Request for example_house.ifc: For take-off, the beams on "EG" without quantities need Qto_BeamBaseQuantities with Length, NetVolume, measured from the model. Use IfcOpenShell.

First a look at what the model holds.

```python
import ifcopenshell
import ifcopenshell.util.element
import ifcopenshell.util.unit

model = ifcopenshell.open("example_house.ifc")
print(model.schema)
for unit_type in ("LENGTHUNIT", "AREAUNIT", "VOLUMEUNIT"):
    print(unit_type, ifcopenshell.util.unit.calculate_unit_scale(model, unit_type))
storey = next(s for s in model.by_type("IfcBuildingStorey") if s.Name == "EG")
beams = [e for e in ifcopenshell.util.element.get_decomposition(storey) if e.is_a("IfcBeam")]
for e in sorted(beams, key=lambda e: e.id()):
    print(e.id(), e.is_a(), e.Name, list(ifcopenshell.util.element.get_psets(e, qtos_only=True)), sep=" | ")
```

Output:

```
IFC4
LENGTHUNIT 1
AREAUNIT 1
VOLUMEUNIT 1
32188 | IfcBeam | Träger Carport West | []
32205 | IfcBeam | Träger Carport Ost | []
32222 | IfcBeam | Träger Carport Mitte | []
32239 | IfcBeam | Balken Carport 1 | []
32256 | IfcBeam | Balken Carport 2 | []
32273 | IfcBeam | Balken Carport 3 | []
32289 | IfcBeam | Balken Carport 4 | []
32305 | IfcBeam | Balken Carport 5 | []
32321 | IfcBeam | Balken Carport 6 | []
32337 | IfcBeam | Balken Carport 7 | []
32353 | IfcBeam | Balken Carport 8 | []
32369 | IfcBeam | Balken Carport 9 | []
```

```python
import ifcopenshell
import ifcopenshell.api.pset
import ifcopenshell.geom
import ifcopenshell.util.element
import ifcopenshell.util.shape
import ifcopenshell.util.unit

model = ifcopenshell.open("example_house.ifc")
unit_scale = ifcopenshell.util.unit.calculate_unit_scale(model)
volume_scale = ifcopenshell.util.unit.calculate_unit_scale(model, "VOLUMEUNIT")
settings = ifcopenshell.geom.settings()

storey = next(s for s in model.by_type("IfcBuildingStorey") if s.Name == "EG")
beams = [e for e in ifcopenshell.util.element.get_decomposition(storey) if e.is_a("IfcBeam")]

for e in sorted(beams, key=lambda e: e.id()):
    if ifcopenshell.util.element.get_psets(e, qtos_only=True, should_inherit=False):
        continue
    # Geometry comes back in metres, in the element's own axes.
    shape = ifcopenshell.geom.create_shape(settings, e)
    values = {
        "Length": ifcopenshell.util.shape.get_max_xyz(shape.geometry) / unit_scale,
        "NetVolume": ifcopenshell.util.shape.get_volume(shape.geometry) / volume_scale,
    }
    qto = ifcopenshell.api.pset.add_qto(model, product=e, name="Qto_BeamBaseQuantities")
    ifcopenshell.api.pset.edit_qto(model, qto=qto, properties=values)
    print(e.id(), {k: round(v, 3) for k, v in values.items()})

model.write("example_house_rev.ifc")
```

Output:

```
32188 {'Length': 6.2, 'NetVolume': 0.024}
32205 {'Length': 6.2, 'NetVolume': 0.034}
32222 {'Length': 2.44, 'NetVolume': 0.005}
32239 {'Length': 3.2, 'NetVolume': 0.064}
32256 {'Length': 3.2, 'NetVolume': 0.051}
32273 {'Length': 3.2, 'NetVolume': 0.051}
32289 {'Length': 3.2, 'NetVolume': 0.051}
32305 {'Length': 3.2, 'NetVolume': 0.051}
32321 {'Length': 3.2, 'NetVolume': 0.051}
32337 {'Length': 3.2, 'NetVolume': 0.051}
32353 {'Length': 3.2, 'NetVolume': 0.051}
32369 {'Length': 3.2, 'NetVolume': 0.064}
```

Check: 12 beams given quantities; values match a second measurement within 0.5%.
